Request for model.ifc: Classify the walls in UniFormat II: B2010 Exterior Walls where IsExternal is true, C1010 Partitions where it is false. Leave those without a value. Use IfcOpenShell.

First a look at what the model holds.

```python
import ifcopenshell
import ifcopenshell.util.element

model = ifcopenshell.open("model.ifc")
print(model.schema)
print("classifications:", [c.Name for c in model.by_type("IfcClassification")])
values = [ifcopenshell.util.element.get_pset(e, "Pset_WallCommon", "IsExternal") for e in model.by_type("IfcWall")]
for value in (True, False, None):
    print("IsExternal", value, values.count(value))
```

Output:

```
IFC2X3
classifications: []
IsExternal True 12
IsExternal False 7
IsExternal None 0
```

```python
import ifcopenshell
import ifcopenshell.api.classification
import ifcopenshell.util.element

model = ifcopenshell.open("model.ifc")

# IFC2X3 requires Source and Edition and has no link from the project to the system.
system = model.create_entity("IfcClassification", Source="ASTM", Edition="E1557", Name="UniFormat II")

walls = model.by_type("IfcWall")
external = {e: ifcopenshell.util.element.get_pset(e, "Pset_WallCommon", "IsExternal") for e in walls}
for flag, code, name in ((True, "B2010", "Exterior Walls"), (False, "C1010", "Partitions")):
    products = [e for e in walls if external[e] is flag]
    ifcopenshell.api.classification.add_reference(
        model, products=products, classification=system, identification=code, name=name
    )
    print(code, len(products))

model.write("model-out.ifc")
```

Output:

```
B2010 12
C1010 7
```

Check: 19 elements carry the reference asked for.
